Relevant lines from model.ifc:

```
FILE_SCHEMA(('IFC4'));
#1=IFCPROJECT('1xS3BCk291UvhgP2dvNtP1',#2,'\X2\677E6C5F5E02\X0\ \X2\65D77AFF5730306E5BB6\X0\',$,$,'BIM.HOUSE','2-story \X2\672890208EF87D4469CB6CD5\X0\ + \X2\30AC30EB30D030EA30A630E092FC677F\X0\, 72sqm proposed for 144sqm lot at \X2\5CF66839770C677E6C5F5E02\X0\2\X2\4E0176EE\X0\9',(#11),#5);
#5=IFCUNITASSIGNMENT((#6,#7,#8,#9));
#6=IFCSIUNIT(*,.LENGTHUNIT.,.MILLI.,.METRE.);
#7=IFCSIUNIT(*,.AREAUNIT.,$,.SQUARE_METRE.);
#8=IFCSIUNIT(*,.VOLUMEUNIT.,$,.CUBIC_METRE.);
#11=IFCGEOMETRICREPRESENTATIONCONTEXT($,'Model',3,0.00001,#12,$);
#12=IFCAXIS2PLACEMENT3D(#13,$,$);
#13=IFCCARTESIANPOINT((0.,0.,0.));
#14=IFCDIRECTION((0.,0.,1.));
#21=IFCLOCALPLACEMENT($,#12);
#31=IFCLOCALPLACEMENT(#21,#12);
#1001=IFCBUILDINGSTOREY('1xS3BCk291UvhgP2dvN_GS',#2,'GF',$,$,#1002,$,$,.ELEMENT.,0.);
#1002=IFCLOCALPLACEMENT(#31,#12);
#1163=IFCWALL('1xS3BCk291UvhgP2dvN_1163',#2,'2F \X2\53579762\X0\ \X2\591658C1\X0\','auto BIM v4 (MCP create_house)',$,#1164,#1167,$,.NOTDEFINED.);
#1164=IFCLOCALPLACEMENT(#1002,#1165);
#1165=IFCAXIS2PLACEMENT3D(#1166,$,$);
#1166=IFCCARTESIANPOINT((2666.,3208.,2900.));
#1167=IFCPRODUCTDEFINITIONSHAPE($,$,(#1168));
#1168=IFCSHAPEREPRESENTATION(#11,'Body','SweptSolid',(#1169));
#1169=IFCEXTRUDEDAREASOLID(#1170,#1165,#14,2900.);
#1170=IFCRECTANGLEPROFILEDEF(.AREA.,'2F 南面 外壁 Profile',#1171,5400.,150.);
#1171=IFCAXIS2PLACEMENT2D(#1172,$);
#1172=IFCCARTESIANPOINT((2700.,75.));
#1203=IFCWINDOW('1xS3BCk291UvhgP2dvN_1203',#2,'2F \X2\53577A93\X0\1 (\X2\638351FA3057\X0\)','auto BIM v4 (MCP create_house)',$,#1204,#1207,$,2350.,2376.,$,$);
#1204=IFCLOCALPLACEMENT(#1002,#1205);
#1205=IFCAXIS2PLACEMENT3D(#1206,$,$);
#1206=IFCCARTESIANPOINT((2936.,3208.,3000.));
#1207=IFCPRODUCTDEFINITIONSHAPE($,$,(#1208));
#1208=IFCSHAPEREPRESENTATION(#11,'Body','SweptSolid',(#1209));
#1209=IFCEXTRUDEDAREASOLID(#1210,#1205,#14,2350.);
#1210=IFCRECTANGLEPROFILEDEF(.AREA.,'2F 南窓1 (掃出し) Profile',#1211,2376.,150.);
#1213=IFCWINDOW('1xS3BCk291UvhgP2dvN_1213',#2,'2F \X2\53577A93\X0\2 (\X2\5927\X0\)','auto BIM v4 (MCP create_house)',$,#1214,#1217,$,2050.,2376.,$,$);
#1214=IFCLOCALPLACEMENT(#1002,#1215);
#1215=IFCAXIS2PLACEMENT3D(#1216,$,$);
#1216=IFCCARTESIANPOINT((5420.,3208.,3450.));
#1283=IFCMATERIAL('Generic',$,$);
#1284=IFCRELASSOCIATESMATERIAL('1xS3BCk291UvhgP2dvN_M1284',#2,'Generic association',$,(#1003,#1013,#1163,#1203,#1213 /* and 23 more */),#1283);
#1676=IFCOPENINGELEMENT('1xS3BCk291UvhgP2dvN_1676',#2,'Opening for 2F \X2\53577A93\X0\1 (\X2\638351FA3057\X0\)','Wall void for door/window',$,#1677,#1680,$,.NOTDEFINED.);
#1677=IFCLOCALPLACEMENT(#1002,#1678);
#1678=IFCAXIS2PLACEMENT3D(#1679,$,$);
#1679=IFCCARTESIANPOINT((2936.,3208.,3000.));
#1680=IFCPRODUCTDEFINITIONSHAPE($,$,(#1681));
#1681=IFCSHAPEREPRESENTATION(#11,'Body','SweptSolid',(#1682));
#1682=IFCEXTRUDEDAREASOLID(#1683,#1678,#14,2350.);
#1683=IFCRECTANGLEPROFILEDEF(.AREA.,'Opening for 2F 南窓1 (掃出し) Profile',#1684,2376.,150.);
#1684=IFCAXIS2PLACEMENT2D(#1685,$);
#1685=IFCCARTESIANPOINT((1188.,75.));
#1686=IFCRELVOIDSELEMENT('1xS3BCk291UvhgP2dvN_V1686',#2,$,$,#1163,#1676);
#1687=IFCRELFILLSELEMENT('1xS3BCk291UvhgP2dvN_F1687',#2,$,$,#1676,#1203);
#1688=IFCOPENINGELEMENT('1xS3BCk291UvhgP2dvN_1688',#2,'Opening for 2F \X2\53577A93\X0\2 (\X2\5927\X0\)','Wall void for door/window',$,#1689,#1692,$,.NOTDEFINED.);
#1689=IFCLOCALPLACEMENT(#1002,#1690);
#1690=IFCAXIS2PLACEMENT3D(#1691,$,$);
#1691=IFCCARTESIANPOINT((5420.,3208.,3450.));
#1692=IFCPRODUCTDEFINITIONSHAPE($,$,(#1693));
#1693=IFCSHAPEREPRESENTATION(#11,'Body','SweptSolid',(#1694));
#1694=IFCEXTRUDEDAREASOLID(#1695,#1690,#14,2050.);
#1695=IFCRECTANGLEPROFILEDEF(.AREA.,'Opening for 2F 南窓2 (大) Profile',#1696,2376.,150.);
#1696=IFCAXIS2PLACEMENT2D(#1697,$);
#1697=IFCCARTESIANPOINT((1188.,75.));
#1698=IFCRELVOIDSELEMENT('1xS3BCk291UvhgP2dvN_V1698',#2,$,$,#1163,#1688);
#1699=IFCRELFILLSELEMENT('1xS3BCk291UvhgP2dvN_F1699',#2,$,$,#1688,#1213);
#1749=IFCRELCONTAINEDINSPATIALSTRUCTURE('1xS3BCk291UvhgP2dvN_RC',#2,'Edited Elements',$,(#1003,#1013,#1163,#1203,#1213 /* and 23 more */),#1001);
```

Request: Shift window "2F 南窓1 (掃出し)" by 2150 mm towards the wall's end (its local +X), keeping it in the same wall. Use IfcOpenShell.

```python
import ifcopenshell
import ifcopenshell.api.geometry
import ifcopenshell.util.placement
import ifcopenshell.util.unit

model = ifcopenshell.open("model.ifc")
unit_scale = ifcopenshell.util.unit.calculate_unit_scale(model)

window = model.by_guid("1xS3BCk291UvhgP2dvN_1203")
opening = window.FillsVoids[0].RelatingOpeningElement
wall = opening.VoidsElements[0].RelatingBuildingElement

wall_matrix = ifcopenshell.util.placement.get_local_placement(wall.ObjectPlacement)
shift = wall_matrix[:3, 0] * 2.15 / unit_scale
before = ifcopenshell.util.placement.get_local_placement(window.ObjectPlacement)[:3, 3].copy()

# The window is not placed relative to its opening, so move both.
for product in (opening, window):
    matrix = ifcopenshell.util.placement.get_local_placement(product.ObjectPlacement)
    matrix[:3, 3] += shift
    ifcopenshell.api.geometry.edit_object_placement(model, product=product, matrix=matrix, is_si=False)

after = ifcopenshell.util.placement.get_local_placement(window.ObjectPlacement)[:3, 3]
print("window moved by", (after - before).round(3) + 0.0)

model.write("model-out.ifc")
```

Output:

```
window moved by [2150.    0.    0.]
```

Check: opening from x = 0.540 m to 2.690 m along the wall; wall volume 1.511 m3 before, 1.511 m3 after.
